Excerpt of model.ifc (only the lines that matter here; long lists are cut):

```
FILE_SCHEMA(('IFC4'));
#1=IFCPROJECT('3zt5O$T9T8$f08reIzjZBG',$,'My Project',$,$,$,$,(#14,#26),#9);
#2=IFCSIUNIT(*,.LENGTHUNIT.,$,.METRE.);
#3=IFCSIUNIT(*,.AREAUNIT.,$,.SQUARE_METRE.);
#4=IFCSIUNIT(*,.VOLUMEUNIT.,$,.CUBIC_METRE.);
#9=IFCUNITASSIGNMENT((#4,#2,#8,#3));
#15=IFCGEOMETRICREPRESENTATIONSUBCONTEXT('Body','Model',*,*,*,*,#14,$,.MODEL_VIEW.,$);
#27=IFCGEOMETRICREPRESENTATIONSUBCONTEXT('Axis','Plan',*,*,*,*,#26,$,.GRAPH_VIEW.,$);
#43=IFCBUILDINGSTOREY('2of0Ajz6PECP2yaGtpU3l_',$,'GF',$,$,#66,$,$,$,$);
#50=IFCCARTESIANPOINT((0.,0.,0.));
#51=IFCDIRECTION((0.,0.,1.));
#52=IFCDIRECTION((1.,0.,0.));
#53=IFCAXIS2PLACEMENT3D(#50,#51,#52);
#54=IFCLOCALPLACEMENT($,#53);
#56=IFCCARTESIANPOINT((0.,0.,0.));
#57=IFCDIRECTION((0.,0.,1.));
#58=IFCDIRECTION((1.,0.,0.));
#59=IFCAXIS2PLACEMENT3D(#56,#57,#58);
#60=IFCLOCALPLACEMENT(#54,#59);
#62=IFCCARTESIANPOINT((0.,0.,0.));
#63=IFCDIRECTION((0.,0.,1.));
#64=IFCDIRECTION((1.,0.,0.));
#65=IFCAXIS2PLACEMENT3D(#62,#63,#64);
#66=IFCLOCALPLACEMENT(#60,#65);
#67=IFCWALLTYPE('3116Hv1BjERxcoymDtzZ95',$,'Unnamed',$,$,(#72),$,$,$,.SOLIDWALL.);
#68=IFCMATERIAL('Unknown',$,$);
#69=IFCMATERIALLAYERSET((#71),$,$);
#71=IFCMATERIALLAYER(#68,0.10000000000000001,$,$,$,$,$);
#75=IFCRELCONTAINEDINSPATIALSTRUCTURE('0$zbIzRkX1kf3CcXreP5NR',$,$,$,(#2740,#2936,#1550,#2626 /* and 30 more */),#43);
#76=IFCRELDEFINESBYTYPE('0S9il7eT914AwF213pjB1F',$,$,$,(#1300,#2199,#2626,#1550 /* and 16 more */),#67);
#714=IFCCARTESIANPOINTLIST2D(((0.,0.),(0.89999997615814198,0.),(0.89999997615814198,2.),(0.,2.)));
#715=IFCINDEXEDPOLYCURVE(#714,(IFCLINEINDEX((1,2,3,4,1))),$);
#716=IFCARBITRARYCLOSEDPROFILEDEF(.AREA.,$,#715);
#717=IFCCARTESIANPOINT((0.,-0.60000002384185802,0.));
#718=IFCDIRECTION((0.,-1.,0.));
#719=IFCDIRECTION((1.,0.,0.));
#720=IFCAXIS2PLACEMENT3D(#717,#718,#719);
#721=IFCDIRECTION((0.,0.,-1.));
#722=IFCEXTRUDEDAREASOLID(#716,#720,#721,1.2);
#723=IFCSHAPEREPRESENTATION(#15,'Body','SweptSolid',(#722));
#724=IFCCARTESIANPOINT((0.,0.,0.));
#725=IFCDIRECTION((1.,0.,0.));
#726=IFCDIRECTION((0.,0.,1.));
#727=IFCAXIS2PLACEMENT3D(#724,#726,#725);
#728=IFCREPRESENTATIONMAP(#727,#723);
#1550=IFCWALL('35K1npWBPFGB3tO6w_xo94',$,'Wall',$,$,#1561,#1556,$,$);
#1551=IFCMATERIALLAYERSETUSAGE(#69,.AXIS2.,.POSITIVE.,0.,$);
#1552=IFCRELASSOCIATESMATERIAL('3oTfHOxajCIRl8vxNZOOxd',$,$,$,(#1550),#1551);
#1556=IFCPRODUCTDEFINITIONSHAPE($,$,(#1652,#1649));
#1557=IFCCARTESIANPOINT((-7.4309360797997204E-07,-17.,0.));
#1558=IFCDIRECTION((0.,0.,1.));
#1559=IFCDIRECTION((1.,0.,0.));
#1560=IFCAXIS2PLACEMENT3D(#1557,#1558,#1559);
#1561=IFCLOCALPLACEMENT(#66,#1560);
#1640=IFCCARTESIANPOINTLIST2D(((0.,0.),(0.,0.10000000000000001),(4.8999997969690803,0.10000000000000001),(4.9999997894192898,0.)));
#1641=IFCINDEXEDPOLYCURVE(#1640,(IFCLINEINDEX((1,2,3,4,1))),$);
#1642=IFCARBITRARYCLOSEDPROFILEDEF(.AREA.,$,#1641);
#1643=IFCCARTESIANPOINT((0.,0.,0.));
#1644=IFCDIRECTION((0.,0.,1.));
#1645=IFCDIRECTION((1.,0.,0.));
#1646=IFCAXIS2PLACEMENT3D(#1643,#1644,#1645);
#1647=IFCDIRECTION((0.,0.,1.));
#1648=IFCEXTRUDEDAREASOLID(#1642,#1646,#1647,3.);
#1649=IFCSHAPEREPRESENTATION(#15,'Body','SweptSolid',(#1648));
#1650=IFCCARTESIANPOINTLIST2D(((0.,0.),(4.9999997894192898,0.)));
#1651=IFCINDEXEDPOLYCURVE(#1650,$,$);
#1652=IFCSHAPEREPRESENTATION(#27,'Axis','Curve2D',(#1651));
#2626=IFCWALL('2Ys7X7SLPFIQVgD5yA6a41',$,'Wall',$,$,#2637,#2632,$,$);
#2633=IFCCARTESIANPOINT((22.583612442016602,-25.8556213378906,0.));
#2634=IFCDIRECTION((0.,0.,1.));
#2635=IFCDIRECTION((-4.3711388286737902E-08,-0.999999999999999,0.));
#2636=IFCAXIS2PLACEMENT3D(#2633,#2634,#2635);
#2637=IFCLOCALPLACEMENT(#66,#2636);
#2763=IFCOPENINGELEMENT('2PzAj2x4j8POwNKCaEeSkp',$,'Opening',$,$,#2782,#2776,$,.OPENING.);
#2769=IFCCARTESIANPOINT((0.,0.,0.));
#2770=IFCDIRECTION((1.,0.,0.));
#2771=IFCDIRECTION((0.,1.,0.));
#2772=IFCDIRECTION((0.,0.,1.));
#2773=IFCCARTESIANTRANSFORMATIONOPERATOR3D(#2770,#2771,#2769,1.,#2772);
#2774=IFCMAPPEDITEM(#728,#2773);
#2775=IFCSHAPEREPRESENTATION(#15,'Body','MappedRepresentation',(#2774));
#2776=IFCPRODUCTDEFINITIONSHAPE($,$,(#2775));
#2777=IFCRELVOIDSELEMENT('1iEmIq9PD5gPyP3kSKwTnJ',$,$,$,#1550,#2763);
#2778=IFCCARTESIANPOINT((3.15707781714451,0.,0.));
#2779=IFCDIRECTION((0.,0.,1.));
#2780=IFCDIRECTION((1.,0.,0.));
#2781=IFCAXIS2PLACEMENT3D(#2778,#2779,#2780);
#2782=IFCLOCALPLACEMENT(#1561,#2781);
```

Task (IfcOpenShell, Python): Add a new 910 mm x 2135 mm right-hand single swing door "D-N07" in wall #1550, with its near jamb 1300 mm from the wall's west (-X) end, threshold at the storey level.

```python
import numpy as np
import ifcopenshell
import ifcopenshell.api.feature
import ifcopenshell.api.geometry
import ifcopenshell.api.root
import ifcopenshell.api.spatial
import ifcopenshell.geom
import ifcopenshell.util.element
import ifcopenshell.util.placement
import ifcopenshell.util.representation
import ifcopenshell.util.shape
import ifcopenshell.util.unit

model = ifcopenshell.open("model.ifc")
unit_scale = ifcopenshell.util.unit.calculate_unit_scale(model)
settings = ifcopenshell.geom.settings()


def volume(element):
    """Net volume in cubic metres, openings subtracted."""
    shape = ifcopenshell.geom.create_shape(settings, element)
    return ifcopenshell.util.shape.get_volume(shape.geometry)


wall = model.by_guid("35K1npWBPFGB3tO6w_xo94")
storey = ifcopenshell.util.element.get_container(wall, ifc_class="IfcBuildingStorey")
context = ifcopenshell.util.representation.get_context(model, "Model", "Body", "MODEL_VIEW")
before = volume(wall)

width, height, from_end, sill = 0.91, 2.135, 1.3, 0.0  # metres

# The wall runs along its own X axis, and the end named is its -X end.
wall_shape = ifcopenshell.geom.create_shape(settings, wall)
x, y, z = ifcopenshell.util.shape.get_vertices(wall_shape.geometry).T
start = x.min() + from_end
face, thickness = float(y.min()), float(y.max() - y.min())
wall_matrix = ifcopenshell.util.placement.get_local_placement(wall.ObjectPlacement)
level = ifcopenshell.util.placement.get_local_placement(storey.ObjectPlacement)[2, 3]


def in_wall(x, y):
    """Placement at x, y metres in the wall's axes, at sill height."""
    matrix = wall_matrix.copy()
    matrix[:, 3] = wall_matrix @ np.array([x / unit_scale, y / unit_scale, 0.0, 1.0])
    matrix[2, 3] = level + sill / unit_scale
    return matrix


# Opening: a box that overshoots both wall faces by 50 mm.
opening = ifcopenshell.api.root.create_entity(model, ifc_class="IfcOpeningElement", predefined_type="OPENING")
box = ifcopenshell.api.geometry.add_wall_representation(
    model, context=context, length=width, height=height, thickness=thickness + 0.1
)
ifcopenshell.api.geometry.assign_representation(model, product=opening, representation=box)
ifcopenshell.api.geometry.edit_object_placement(model, product=opening, matrix=in_wall(start, face - 0.05), is_si=False)
ifcopenshell.api.feature.add_feature(model, feature=opening, element=wall)

door = ifcopenshell.api.root.create_entity(model, ifc_class="IfcDoor", name="D-N07", predefined_type="DOOR")
door.OverallWidth, door.OverallHeight = width / unit_scale, height / unit_scale
door.OperationType = "SINGLE_SWING_RIGHT"
body = ifcopenshell.api.geometry.add_door_representation(
    model,
    context=context,
    overall_width=door.OverallWidth,
    overall_height=door.OverallHeight,
    operation_type="SINGLE_SWING_RIGHT",
    lining_properties={"LiningDepth": thickness / unit_scale, "ThresholdDepth": thickness / unit_scale},
)
ifcopenshell.api.geometry.assign_representation(model, product=door, representation=body)
ifcopenshell.api.spatial.assign_container(model, products=[door], relating_structure=storey)
ifcopenshell.api.feature.add_filling(model, opening=opening, element=door)

# The lining spans the wall, so the door starts at the wall face.
ifcopenshell.api.geometry.edit_object_placement(model, product=door, matrix=in_wall(start, face), is_si=False)

after = volume(wall)

print(f"wall volume {before:.3f} -> {after:.3f} m3")

model.write("model_updated.ifc")
```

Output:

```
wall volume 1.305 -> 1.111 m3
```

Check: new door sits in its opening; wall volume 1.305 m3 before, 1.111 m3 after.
